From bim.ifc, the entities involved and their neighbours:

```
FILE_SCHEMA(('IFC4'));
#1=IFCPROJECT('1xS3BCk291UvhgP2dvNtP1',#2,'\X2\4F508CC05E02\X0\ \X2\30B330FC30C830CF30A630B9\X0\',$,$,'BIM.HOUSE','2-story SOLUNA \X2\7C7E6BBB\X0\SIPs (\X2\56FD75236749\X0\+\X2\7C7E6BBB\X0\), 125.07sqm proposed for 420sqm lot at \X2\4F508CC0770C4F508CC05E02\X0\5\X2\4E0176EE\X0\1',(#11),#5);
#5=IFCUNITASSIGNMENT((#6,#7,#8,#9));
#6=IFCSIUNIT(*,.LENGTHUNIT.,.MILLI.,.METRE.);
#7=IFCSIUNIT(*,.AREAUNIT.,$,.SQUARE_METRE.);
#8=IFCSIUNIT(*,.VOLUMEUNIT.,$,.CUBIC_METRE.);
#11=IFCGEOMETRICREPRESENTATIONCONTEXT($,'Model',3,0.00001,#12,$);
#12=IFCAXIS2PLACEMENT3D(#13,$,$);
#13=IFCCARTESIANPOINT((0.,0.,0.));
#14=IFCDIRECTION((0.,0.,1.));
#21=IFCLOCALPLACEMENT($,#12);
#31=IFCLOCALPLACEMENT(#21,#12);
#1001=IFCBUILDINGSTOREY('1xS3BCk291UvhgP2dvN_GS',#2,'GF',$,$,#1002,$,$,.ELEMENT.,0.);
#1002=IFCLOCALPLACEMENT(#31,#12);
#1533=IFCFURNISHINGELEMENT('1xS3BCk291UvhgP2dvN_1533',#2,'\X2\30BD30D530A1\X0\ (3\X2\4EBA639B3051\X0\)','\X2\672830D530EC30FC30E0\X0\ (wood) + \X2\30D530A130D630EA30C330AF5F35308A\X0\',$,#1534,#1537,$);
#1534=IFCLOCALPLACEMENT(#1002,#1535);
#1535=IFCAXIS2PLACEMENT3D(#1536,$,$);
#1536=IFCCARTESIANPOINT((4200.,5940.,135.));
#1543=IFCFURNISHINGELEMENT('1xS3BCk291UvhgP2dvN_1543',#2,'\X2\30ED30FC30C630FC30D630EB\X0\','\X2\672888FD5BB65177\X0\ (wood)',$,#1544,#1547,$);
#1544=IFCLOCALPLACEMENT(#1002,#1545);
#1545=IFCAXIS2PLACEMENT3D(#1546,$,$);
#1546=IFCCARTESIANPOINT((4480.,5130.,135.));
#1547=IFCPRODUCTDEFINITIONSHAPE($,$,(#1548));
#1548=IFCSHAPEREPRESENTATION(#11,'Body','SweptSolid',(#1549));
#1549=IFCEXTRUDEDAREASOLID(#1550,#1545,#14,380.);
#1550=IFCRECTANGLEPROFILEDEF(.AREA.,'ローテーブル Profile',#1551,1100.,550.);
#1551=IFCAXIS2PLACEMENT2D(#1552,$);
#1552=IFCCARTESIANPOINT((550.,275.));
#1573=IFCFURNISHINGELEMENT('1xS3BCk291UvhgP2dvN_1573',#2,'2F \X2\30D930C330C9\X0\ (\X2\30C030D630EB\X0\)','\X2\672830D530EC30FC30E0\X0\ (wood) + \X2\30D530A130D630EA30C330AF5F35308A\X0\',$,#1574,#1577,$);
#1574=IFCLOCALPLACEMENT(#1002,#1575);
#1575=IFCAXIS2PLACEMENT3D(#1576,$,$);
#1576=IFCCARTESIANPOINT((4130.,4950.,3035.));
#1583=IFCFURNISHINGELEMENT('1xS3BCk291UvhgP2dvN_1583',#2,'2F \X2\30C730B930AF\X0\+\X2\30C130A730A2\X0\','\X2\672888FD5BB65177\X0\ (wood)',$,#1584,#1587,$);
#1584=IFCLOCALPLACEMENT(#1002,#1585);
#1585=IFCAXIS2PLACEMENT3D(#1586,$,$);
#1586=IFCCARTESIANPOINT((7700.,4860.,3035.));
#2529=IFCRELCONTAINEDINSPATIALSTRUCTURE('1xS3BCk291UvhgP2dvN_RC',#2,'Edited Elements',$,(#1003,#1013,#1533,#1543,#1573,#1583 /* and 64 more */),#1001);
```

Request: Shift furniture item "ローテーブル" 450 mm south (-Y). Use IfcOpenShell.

```python
import ifcopenshell
import ifcopenshell.api.geometry
import ifcopenshell.util.placement

model = ifcopenshell.open("bim.ifc")

item = model.by_id(1543)
matrix = ifcopenshell.util.placement.get_local_placement(item.ObjectPlacement)
matrix[1, 3] -= 450.0
ifcopenshell.api.geometry.edit_object_placement(model, product=item, matrix=matrix, is_si=False)

print(ifcopenshell.util.placement.get_local_placement(item.ObjectPlacement).round(3) + 0.0)

model.write("bim_v2.ifc")
```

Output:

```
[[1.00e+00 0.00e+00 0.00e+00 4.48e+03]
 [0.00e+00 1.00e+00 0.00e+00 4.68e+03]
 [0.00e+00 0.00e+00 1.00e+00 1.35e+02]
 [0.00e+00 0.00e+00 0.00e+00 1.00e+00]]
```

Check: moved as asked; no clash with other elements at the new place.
